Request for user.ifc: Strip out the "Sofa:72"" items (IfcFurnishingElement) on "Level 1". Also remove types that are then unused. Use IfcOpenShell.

First a look at what the model holds.

```python
import ifcopenshell
import ifcopenshell.util.element

model = ifcopenshell.open("user.ifc")
print(model.schema)
storey = next(s for s in model.by_type("IfcBuildingStorey") if s.Name == "Level 1")
furniture = [e for e in ifcopenshell.util.element.get_decomposition(storey) if e.is_a("IfcFurnishingElement")]
seen = {}
for e in furniture:
    element_type = ifcopenshell.util.element.get_type(e)
    name = element_type.Name if element_type not in (None, e) else None
    seen[name] = seen.get(name, 0) + 1
for name, count in sorted(seen.items(), key=str):
    print(count, "x", name)
```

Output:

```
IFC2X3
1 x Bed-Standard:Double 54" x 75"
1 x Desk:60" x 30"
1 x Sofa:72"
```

```python
import ifcopenshell
import ifcopenshell.api.root
import ifcopenshell.util.element

model = ifcopenshell.open("user.ifc")

storey = next(s for s in model.by_type("IfcBuildingStorey") if s.Name == "Level 1")
furniture = [e for e in ifcopenshell.util.element.get_decomposition(storey) if e.is_a("IfcFurnishingElement")]
targets = [e for e in furniture if (t := ifcopenshell.util.element.get_type(e)) not in (None, e) and t.Name == 'Sofa:72"']
types = {ifcopenshell.util.element.get_type(e) for e in targets} - {None, *targets}

for e in targets:
    ifcopenshell.api.root.remove_product(model, product=e)
print(len(targets), "removed")

unused = [t for t in types if not ifcopenshell.util.element.get_types(t)]
for t in unused:
    ifcopenshell.api.root.remove_product(model, product=t)
print(len(unused), "unused types removed")

model.write("user_rev.ifc")
```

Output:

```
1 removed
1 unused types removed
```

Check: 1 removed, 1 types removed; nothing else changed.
